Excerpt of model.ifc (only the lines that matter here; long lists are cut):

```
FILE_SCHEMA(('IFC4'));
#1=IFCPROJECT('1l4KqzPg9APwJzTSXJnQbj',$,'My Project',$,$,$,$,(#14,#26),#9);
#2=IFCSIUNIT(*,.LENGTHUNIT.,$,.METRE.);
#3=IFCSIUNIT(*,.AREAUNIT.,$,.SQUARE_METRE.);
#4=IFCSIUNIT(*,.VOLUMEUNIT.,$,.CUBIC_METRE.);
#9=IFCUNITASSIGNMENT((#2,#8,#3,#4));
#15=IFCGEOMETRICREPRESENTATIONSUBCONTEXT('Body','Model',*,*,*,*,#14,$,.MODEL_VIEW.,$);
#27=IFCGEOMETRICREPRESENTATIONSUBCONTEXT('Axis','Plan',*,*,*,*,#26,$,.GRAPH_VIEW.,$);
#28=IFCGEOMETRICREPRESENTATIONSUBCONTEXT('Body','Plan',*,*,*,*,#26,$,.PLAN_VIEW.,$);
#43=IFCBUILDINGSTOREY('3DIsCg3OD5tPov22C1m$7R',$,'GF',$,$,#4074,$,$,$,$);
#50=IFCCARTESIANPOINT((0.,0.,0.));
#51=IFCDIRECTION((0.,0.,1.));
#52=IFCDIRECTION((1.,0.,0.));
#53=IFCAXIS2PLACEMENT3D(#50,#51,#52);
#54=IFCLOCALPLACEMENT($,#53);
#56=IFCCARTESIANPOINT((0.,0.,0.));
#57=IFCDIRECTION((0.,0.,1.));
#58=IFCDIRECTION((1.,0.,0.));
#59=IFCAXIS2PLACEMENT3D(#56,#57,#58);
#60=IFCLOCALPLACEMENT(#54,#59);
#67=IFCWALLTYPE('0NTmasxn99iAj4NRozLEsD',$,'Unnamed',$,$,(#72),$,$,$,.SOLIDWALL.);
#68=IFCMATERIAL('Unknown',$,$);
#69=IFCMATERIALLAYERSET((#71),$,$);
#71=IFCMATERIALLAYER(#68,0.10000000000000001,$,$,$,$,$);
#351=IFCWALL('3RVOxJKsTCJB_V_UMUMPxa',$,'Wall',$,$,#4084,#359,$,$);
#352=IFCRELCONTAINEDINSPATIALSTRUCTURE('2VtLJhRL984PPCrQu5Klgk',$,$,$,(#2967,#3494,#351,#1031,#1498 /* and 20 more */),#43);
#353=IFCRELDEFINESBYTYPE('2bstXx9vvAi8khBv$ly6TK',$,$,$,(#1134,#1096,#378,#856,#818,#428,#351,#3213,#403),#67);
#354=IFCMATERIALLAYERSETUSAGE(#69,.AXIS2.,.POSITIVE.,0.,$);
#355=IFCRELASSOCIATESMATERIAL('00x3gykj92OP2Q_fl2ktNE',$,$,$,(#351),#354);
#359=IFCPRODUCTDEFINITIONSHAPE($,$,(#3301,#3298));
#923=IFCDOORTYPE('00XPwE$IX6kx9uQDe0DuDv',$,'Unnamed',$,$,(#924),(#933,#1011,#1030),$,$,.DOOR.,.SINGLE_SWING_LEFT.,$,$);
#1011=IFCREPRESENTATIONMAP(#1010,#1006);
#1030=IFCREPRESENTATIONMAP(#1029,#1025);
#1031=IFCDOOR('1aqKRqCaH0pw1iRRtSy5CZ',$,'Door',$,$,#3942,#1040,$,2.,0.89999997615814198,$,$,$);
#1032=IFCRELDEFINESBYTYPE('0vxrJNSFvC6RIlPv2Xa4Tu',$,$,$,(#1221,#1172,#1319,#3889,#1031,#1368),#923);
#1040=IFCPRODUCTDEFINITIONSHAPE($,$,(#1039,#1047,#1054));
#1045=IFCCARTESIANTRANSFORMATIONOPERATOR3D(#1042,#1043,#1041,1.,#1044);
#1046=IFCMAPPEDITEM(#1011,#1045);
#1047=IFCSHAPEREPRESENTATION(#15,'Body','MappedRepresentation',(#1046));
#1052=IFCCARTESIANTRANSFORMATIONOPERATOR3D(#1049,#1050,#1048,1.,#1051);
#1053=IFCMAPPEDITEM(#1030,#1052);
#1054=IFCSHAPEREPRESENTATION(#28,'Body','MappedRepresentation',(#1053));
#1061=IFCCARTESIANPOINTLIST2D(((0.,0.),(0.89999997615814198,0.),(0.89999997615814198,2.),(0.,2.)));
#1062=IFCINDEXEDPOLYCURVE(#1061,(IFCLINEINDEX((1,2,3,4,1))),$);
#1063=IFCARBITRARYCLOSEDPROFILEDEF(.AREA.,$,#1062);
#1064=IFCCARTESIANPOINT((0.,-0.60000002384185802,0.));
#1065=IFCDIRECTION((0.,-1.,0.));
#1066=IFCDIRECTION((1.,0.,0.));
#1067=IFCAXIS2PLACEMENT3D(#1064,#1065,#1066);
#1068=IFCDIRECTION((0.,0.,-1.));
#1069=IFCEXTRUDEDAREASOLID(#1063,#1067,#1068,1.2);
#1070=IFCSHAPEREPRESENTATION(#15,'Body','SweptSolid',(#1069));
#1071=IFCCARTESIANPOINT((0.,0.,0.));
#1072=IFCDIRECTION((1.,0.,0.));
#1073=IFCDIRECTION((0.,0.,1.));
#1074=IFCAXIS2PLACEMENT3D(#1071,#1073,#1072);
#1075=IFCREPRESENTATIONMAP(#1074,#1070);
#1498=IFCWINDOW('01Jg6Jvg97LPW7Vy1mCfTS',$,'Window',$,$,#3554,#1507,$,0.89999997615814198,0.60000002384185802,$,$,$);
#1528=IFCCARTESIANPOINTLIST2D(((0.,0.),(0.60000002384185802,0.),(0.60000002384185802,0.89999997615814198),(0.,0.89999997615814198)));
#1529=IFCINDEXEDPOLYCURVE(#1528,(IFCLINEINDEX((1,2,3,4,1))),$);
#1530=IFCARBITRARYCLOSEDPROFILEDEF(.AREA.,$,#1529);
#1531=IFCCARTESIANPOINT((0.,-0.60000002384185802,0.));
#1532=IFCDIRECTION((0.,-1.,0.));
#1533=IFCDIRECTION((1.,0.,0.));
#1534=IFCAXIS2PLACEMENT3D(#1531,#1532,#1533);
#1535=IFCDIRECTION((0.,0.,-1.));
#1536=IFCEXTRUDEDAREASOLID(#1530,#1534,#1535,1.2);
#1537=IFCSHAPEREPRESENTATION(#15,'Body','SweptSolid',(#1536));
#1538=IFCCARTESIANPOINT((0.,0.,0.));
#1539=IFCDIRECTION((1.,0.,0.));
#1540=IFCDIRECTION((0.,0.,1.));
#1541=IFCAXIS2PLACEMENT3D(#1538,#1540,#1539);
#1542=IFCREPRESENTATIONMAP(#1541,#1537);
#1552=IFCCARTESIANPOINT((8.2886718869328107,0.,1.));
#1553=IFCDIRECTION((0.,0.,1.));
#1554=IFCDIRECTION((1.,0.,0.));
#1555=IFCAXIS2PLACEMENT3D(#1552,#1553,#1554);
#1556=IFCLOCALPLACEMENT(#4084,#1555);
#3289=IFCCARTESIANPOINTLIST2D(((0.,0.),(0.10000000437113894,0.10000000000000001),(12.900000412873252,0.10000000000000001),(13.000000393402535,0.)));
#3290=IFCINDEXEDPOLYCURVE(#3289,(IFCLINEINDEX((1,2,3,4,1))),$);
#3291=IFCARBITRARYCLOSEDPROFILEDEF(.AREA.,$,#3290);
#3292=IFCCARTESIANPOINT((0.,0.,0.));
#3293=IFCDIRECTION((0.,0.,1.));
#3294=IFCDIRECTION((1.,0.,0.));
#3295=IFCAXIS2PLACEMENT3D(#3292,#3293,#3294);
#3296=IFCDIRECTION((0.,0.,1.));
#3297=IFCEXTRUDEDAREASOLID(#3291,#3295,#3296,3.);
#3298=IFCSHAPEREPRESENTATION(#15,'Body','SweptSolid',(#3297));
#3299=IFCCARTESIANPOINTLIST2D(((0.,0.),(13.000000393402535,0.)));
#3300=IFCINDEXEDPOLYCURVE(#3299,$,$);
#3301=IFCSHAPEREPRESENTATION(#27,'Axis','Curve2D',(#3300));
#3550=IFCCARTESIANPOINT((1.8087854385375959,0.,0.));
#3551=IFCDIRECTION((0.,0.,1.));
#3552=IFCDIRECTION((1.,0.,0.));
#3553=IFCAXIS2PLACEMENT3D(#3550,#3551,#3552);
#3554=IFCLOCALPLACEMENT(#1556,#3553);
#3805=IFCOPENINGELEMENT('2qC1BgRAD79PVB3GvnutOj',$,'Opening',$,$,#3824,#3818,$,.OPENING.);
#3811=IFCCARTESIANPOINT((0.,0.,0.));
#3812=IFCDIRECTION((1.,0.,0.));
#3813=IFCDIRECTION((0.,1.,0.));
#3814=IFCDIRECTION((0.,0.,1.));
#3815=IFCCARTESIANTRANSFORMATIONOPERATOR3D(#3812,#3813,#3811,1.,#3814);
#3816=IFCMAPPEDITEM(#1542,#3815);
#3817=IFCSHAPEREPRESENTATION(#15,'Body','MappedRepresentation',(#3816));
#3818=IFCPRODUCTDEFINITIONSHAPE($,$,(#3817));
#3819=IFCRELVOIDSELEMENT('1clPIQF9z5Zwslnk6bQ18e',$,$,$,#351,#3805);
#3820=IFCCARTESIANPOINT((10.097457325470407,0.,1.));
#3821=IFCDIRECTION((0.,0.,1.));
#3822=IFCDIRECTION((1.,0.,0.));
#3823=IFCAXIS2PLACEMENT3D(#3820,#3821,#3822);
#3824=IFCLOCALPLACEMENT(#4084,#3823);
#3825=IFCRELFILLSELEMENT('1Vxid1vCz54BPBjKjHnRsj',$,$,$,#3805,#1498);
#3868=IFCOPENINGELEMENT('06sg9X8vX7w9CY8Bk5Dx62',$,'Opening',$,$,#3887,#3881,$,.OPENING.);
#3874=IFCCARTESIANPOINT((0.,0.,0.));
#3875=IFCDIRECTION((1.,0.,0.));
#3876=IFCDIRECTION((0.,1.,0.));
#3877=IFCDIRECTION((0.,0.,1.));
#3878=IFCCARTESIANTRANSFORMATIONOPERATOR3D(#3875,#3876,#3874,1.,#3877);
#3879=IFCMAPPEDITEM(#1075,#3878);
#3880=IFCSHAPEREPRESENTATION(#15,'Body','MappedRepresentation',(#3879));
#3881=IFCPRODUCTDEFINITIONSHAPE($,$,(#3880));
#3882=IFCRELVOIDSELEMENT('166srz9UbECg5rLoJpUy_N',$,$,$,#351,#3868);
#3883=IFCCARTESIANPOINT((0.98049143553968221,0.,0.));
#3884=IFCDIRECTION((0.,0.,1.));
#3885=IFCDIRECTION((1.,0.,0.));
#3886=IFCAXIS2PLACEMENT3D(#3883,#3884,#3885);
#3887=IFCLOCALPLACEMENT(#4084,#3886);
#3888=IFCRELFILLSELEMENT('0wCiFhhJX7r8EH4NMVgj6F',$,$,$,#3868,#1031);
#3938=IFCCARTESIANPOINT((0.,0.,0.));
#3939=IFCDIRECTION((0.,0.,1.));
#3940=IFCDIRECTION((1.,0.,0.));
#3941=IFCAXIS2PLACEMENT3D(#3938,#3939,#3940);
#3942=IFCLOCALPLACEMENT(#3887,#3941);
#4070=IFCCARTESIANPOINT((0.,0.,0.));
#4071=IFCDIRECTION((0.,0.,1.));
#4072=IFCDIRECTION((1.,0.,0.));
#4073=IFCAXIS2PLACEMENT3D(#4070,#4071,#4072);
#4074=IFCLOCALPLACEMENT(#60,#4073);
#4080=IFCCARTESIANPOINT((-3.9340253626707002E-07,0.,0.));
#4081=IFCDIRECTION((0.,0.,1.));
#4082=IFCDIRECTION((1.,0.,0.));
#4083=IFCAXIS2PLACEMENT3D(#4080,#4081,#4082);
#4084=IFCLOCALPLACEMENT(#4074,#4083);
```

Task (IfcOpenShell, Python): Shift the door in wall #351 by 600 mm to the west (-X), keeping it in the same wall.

```python
import ifcopenshell
import ifcopenshell.api.geometry
import ifcopenshell.util.placement
import ifcopenshell.util.unit

model = ifcopenshell.open("model.ifc")
unit_scale = ifcopenshell.util.unit.calculate_unit_scale(model)

door = model.by_guid("1aqKRqCaH0pw1iRRtSy5CZ")
opening = door.FillsVoids[0].RelatingOpeningElement
wall = opening.VoidsElements[0].RelatingBuildingElement

wall_matrix = ifcopenshell.util.placement.get_local_placement(wall.ObjectPlacement)
shift = wall_matrix[:3, 0] * -0.6 / unit_scale
before = ifcopenshell.util.placement.get_local_placement(door.ObjectPlacement)[:3, 3].copy()

# The door is placed relative to its opening, so it follows when the opening moves.
matrix = ifcopenshell.util.placement.get_local_placement(opening.ObjectPlacement)
matrix[:3, 3] += shift
ifcopenshell.api.geometry.edit_object_placement(
    model, product=opening, matrix=matrix, is_si=False, should_transform_children=True
)

after = ifcopenshell.util.placement.get_local_placement(door.ObjectPlacement)[:3, 3]
print("door moved by", (after - before).round(3) + 0.0)

model.write("model-out.ifc")
```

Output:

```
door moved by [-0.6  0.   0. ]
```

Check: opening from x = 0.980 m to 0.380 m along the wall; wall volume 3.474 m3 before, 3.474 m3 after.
